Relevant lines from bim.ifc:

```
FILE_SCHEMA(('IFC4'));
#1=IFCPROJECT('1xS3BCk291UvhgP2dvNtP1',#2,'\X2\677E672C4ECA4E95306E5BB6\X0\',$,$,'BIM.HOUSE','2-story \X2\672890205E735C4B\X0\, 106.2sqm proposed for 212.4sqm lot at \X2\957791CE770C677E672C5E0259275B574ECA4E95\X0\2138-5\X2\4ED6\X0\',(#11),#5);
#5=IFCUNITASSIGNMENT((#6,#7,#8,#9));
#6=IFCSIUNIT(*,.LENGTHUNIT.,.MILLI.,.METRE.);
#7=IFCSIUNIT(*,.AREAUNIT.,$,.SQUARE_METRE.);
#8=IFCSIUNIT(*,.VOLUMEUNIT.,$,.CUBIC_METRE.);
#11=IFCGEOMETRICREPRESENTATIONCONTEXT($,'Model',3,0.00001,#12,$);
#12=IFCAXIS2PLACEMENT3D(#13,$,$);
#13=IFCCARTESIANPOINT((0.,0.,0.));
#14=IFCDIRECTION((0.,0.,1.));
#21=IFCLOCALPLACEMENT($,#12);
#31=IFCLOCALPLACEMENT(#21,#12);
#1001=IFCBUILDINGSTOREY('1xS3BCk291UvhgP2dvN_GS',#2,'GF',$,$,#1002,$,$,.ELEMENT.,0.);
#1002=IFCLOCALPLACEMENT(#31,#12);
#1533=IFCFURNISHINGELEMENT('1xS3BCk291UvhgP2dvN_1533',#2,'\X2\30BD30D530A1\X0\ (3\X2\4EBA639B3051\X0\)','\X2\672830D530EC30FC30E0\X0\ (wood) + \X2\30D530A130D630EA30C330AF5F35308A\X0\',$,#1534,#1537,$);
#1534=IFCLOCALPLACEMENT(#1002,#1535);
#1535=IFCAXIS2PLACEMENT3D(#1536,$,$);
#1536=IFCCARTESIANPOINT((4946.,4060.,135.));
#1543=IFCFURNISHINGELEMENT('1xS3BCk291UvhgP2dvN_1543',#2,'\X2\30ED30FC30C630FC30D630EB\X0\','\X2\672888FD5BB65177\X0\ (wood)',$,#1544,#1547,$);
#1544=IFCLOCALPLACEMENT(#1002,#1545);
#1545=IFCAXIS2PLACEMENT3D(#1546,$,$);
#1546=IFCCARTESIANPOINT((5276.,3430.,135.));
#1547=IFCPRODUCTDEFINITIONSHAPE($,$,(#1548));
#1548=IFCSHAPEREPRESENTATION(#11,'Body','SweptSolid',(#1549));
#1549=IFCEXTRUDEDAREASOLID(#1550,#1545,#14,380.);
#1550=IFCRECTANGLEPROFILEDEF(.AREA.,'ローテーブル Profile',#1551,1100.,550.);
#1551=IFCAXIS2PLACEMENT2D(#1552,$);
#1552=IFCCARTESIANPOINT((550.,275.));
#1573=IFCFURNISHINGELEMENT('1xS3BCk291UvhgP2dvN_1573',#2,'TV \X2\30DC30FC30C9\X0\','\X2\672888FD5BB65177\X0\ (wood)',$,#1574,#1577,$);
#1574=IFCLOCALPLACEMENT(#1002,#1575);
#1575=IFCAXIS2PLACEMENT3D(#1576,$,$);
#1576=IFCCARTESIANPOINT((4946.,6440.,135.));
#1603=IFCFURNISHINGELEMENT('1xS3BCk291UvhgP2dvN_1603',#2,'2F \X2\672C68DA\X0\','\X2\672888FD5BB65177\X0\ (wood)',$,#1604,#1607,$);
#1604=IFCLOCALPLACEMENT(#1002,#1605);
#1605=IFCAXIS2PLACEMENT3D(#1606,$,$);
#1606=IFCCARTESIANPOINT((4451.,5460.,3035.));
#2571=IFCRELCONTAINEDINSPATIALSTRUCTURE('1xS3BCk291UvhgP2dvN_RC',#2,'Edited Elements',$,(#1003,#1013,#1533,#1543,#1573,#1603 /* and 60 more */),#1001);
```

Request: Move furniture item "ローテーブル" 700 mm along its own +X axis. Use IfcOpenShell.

```python
import ifcopenshell
import ifcopenshell.api.geometry
import ifcopenshell.util.placement

model = ifcopenshell.open("bim.ifc")

item = model.by_id(1543)
matrix = ifcopenshell.util.placement.get_local_placement(item.ObjectPlacement)
matrix[:3, 3] += matrix[:3, 0] * 700.0
ifcopenshell.api.geometry.edit_object_placement(model, product=item, matrix=matrix, is_si=False)

print(ifcopenshell.util.placement.get_local_placement(item.ObjectPlacement).round(3) + 0.0)

model.write("bim_edited.ifc")
```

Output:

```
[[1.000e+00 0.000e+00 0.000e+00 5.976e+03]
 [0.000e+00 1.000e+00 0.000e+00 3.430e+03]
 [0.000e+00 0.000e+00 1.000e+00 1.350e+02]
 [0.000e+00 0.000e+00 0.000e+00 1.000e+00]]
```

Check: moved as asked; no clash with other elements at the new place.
